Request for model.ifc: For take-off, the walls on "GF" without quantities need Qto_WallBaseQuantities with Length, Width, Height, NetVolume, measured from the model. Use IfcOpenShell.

First a look at what the model holds.

```python
import ifcopenshell
import ifcopenshell.util.element
import ifcopenshell.util.unit

model = ifcopenshell.open("model.ifc")
print(model.schema)
for unit_type in ("LENGTHUNIT", "AREAUNIT", "VOLUMEUNIT"):
    print(unit_type, ifcopenshell.util.unit.calculate_unit_scale(model, unit_type))
storey = next(s for s in model.by_type("IfcBuildingStorey") if s.Name == "GF")
walls = [e for e in ifcopenshell.util.element.get_decomposition(storey) if e.is_a("IfcWall")]
for e in sorted(walls, key=lambda e: e.id()):
    print(e.id(), e.is_a(), e.Name, list(ifcopenshell.util.element.get_psets(e, qtos_only=True)), sep=" | ")
```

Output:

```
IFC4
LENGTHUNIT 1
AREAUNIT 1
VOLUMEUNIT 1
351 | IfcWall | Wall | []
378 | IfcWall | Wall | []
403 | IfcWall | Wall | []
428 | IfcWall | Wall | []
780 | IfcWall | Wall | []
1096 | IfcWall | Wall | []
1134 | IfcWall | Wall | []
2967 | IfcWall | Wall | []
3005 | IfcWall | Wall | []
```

```python
import ifcopenshell
import ifcopenshell.api.pset
import ifcopenshell.geom
import ifcopenshell.util.element
import ifcopenshell.util.shape
import ifcopenshell.util.unit

model = ifcopenshell.open("model.ifc")
unit_scale = ifcopenshell.util.unit.calculate_unit_scale(model)
volume_scale = ifcopenshell.util.unit.calculate_unit_scale(model, "VOLUMEUNIT")
settings = ifcopenshell.geom.settings()

storey = next(s for s in model.by_type("IfcBuildingStorey") if s.Name == "GF")
walls = [e for e in ifcopenshell.util.element.get_decomposition(storey) if e.is_a("IfcWall")]

for e in sorted(walls, key=lambda e: e.id()):
    if ifcopenshell.util.element.get_psets(e, qtos_only=True, should_inherit=False):
        continue
    # Geometry comes back in metres, in the element's own axes.
    shape = ifcopenshell.geom.create_shape(settings, e)
    values = {
        "Length": ifcopenshell.util.shape.get_x(shape.geometry) / unit_scale,
        "Width": ifcopenshell.util.shape.get_y(shape.geometry) / unit_scale,
        "Height": ifcopenshell.util.shape.get_z(shape.geometry) / unit_scale,
        "NetVolume": ifcopenshell.util.shape.get_volume(shape.geometry) / volume_scale,
    }
    qto = ifcopenshell.api.pset.add_qto(model, product=e, name="Qto_WallBaseQuantities")
    ifcopenshell.api.pset.edit_qto(model, qto=qto, properties=values)
    print(e.id(), {k: round(v, 3) for k, v in values.items()})

model.write("model_edited.ifc")
```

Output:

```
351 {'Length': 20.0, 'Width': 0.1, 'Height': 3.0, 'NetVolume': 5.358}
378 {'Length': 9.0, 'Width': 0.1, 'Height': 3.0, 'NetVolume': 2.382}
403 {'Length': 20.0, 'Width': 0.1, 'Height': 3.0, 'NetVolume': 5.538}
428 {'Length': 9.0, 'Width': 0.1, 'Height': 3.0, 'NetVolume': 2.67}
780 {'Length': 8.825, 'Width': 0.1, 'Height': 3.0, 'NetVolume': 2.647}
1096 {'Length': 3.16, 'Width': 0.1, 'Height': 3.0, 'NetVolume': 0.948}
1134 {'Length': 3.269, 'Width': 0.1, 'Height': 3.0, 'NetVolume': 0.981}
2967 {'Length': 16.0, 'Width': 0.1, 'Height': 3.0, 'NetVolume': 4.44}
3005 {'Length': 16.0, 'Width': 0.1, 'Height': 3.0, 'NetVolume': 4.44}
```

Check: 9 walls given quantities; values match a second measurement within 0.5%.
